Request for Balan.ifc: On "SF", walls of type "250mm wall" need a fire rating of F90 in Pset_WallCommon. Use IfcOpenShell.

First a look at what the model holds.

```python
import ifcopenshell
import ifcopenshell.util.element

model = ifcopenshell.open("Balan.ifc")
print(model.schema)
storey = next(s for s in model.by_type("IfcBuildingStorey") if s.Name == "SF")
walls = [e for e in ifcopenshell.util.element.get_decomposition(storey) if e.is_a("IfcWall")]
seen = {}
for e in walls:
    element_type = ifcopenshell.util.element.get_type(e)
    key = (element_type.Name if element_type != e and element_type else None, ifcopenshell.util.element.get_pset(e, "Pset_WallCommon", "FireRating"))
    seen[key] = seen.get(key, 0) + 1
for (name, value), count in sorted(seen.items(), key=str):
    print(count, "x", name, "|", value)
```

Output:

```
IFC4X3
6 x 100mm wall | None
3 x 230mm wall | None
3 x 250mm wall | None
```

```python
import ifcopenshell
import ifcopenshell.api.pset
import ifcopenshell.util.element

model = ifcopenshell.open("Balan.ifc")

storey = next(s for s in model.by_type("IfcBuildingStorey") if s.Name == "SF")
walls = [e for e in ifcopenshell.util.element.get_decomposition(storey) if e.is_a("IfcWall")]

count = 0
for e in walls:
    element_type = ifcopenshell.util.element.get_type(e)
    if element_type in (None, e) or element_type.Name != "250mm wall":
        continue
    # add_pset returns the element's existing set when there is one.
    pset = ifcopenshell.api.pset.add_pset(model, product=e, name="Pset_WallCommon")
    ifcopenshell.api.pset.edit_pset(model, pset=pset, properties={"FireRating": "F90"})
    count += 1

print(count, "walls updated")

model.write("Balan_rev.ifc")
```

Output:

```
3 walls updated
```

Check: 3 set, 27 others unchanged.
